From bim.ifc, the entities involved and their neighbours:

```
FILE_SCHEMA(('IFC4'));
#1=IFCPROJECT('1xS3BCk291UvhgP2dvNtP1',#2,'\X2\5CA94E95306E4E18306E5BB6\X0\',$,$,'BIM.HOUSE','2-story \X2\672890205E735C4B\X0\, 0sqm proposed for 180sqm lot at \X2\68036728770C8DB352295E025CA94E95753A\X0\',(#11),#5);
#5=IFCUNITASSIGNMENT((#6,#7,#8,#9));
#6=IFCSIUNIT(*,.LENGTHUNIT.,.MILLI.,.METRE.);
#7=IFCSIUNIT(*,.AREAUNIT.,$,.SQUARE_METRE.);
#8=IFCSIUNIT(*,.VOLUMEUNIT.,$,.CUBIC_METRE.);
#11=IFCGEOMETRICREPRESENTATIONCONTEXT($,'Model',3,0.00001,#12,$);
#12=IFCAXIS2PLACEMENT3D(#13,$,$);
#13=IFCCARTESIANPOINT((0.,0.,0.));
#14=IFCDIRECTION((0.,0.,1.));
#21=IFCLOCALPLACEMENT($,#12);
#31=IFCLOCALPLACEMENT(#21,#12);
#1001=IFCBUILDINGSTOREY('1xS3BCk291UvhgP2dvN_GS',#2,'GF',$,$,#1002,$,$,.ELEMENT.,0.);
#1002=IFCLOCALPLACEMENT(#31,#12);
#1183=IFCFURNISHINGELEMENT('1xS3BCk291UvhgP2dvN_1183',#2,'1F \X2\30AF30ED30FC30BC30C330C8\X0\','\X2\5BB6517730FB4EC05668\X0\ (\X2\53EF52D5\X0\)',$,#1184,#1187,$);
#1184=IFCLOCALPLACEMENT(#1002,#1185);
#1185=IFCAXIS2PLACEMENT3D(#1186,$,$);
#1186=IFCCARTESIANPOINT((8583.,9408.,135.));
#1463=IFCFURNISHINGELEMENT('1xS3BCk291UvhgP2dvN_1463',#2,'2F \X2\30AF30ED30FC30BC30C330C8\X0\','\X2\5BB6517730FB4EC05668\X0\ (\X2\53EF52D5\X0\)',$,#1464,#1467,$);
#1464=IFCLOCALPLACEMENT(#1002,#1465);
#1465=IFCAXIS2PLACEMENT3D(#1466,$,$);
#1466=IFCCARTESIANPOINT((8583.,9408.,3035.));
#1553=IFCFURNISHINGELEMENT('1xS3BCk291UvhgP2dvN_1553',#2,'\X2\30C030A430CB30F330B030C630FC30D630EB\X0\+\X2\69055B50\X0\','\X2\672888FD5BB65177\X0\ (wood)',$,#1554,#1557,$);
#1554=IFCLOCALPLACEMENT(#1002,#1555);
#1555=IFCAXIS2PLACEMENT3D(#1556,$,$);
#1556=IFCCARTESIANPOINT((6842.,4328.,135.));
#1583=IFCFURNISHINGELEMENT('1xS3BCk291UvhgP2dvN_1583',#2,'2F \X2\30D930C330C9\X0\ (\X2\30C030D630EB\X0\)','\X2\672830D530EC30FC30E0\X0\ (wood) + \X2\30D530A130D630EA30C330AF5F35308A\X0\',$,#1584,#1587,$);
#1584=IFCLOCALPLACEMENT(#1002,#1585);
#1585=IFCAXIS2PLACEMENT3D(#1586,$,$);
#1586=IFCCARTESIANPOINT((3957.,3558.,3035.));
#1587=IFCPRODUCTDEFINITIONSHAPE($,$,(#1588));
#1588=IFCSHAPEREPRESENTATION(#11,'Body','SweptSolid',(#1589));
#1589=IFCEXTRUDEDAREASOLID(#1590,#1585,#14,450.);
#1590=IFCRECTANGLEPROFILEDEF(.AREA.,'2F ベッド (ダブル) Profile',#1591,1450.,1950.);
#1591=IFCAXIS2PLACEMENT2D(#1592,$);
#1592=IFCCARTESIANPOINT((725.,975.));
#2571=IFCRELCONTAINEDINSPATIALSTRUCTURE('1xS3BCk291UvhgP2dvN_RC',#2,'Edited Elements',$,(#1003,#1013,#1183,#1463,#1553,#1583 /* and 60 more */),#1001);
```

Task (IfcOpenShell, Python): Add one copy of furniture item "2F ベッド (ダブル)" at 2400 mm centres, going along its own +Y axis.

```python
import ifcopenshell
import ifcopenshell.api.geometry
import ifcopenshell.api.root
import ifcopenshell.util.element
import ifcopenshell.util.placement

model = ifcopenshell.open("bim.ifc")


def reuse_history(source, copy):
    """copy_class also copies each property set's owner history, people and application; keep the originals."""
    for rel in copy.IsDefinedBy:
        if rel.is_a("IfcRelDefinesByProperties") and (history := rel.RelatingPropertyDefinition.OwnerHistory):
            rel.RelatingPropertyDefinition.OwnerHistory = source.OwnerHistory
            ifcopenshell.util.element.remove_deep2(model, history)


source = model.by_guid("1xS3BCk291UvhgP2dvN_1583")
base = ifcopenshell.util.placement.get_local_placement(source.ObjectPlacement)
step = base[:3, 1] * 2400.0

for i in range(1, 2):
    copy = ifcopenshell.api.root.copy_class(model, product=source)
    copy.Representation = ifcopenshell.util.element.copy_deep(
        model, source.Representation, exclude=["IfcGeometricRepresentationContext", "IfcRepresentationMap"]
    )
    reuse_history(source, copy)
    matrix = base.copy()
    matrix[:3, 3] += i * step
    print("added at", matrix[:3, 3].round(3) + 0.0)
    ifcopenshell.api.geometry.edit_object_placement(model, product=copy, matrix=matrix, is_si=False)

model.write("bim_edited.ifc")
```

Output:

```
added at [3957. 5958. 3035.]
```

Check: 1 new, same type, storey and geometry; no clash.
